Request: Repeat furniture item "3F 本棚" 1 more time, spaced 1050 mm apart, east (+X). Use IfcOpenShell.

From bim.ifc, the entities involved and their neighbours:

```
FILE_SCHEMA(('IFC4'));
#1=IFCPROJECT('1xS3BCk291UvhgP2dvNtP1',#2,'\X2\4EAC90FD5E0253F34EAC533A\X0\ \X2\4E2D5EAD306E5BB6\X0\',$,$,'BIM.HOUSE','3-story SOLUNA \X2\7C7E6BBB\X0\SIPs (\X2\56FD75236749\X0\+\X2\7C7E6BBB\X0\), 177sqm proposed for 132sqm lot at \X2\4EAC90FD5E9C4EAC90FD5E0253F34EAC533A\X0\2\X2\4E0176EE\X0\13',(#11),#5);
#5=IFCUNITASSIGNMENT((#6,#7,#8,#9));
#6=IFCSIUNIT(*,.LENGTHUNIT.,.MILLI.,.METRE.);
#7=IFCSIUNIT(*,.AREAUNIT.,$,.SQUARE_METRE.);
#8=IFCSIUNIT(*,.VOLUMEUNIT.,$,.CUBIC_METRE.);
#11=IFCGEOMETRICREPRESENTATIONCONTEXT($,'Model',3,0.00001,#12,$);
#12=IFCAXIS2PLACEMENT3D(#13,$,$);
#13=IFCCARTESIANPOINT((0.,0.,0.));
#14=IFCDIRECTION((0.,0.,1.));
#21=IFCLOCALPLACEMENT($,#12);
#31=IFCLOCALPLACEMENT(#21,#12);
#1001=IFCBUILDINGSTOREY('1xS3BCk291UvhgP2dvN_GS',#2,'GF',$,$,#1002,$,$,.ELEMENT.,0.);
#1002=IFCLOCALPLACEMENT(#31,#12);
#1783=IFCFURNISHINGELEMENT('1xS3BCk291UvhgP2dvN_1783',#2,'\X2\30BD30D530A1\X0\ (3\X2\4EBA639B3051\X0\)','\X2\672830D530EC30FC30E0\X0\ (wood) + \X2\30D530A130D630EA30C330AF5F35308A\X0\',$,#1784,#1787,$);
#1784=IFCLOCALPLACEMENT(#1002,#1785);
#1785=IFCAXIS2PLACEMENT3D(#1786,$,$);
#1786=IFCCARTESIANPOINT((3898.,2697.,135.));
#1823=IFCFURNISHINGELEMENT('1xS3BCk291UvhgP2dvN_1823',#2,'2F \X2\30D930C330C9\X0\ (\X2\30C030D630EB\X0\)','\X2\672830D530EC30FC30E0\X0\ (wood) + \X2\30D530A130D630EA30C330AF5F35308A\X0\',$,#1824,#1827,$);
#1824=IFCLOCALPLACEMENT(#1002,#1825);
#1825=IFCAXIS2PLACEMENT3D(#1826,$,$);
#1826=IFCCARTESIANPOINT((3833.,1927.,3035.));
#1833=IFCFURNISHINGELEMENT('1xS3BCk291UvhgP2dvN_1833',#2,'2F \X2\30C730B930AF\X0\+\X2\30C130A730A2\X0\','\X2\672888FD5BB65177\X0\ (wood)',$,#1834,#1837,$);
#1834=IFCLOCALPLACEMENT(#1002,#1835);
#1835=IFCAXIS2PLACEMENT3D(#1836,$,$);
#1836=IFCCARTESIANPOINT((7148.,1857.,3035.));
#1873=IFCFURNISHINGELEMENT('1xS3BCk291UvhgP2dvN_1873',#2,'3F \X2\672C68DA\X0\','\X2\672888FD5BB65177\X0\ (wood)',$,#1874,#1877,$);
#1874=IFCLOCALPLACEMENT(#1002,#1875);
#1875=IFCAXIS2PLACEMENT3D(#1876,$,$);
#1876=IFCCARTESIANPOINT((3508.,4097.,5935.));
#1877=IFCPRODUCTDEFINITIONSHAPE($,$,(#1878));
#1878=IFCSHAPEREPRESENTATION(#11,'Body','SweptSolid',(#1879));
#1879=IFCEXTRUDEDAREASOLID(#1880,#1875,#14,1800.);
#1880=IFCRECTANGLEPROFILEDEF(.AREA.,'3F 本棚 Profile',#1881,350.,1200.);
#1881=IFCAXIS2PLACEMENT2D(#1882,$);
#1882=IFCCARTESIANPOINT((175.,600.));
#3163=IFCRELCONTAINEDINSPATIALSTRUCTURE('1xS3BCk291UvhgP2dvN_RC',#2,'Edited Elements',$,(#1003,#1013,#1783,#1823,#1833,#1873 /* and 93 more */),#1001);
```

```python
import numpy as np
import ifcopenshell
import ifcopenshell.api.geometry
import ifcopenshell.api.root
import ifcopenshell.util.element
import ifcopenshell.util.placement
import ifcopenshell.util.unit

model = ifcopenshell.open("bim.ifc")
unit_scale = ifcopenshell.util.unit.calculate_unit_scale(model)


def reuse_history(source, copy):
    """copy_class also copies each property set's owner history, people and application; keep the originals."""
    for rel in copy.IsDefinedBy:
        if rel.is_a("IfcRelDefinesByProperties") and (history := rel.RelatingPropertyDefinition.OwnerHistory):
            rel.RelatingPropertyDefinition.OwnerHistory = source.OwnerHistory
            ifcopenshell.util.element.remove_deep2(model, history)


source = model.by_guid("1xS3BCk291UvhgP2dvN_1873")
base = ifcopenshell.util.placement.get_local_placement(source.ObjectPlacement)
step = np.array([1.0, 0.0, 0.0]) * 1.05 / unit_scale

for i in range(1, 2):
    copy = ifcopenshell.api.root.copy_class(model, product=source)
    copy.Representation = ifcopenshell.util.element.copy_deep(
        model, source.Representation, exclude=["IfcGeometricRepresentationContext", "IfcRepresentationMap"]
    )
    reuse_history(source, copy)
    matrix = base.copy()
    matrix[:3, 3] += i * step
    print("added at", matrix[:3, 3].round(3) + 0.0)
    ifcopenshell.api.geometry.edit_object_placement(model, product=copy, matrix=matrix, is_si=False)

model.write("bim_edited.ifc")
```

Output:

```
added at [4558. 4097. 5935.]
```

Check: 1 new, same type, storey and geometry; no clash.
